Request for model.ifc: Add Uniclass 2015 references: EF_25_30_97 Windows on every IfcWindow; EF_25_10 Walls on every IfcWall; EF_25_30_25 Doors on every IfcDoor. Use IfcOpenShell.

First a look at what the model holds.

```python
import ifcopenshell

model = ifcopenshell.open("model.ifc")
print(model.schema)
print("classifications:", [c.Name for c in model.by_type("IfcClassification")])
for ifc_class in ("IfcDoor", "IfcRoof", "IfcStair", "IfcWall", "IfcWindow"):
    print(ifc_class, len(model.by_type(ifc_class)))
```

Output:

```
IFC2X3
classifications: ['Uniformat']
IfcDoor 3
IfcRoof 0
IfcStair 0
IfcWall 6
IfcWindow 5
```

```python
import ifcopenshell
import ifcopenshell.api.classification

model = ifcopenshell.open("model.ifc")

# IFC2X3 requires Source and Edition and has no link from the project to the system.
system = model.create_entity("IfcClassification", Source="NBS", Edition="2015", Name="Uniclass 2015")

codes = {
    "IfcWindow": ("EF_25_30_97", "Windows"),
    "IfcWall": ("EF_25_10", "Walls"),
    "IfcDoor": ("EF_25_30_25", "Doors"),
}
for ifc_class, (code, name) in codes.items():
    products = model.by_type(ifc_class)
    ifcopenshell.api.classification.add_reference(
        model, products=products, classification=system, identification=code, name=name
    )
    print(code, len(products))

model.write("model_rev.ifc")
```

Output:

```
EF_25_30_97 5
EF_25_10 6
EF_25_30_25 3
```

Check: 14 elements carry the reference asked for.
